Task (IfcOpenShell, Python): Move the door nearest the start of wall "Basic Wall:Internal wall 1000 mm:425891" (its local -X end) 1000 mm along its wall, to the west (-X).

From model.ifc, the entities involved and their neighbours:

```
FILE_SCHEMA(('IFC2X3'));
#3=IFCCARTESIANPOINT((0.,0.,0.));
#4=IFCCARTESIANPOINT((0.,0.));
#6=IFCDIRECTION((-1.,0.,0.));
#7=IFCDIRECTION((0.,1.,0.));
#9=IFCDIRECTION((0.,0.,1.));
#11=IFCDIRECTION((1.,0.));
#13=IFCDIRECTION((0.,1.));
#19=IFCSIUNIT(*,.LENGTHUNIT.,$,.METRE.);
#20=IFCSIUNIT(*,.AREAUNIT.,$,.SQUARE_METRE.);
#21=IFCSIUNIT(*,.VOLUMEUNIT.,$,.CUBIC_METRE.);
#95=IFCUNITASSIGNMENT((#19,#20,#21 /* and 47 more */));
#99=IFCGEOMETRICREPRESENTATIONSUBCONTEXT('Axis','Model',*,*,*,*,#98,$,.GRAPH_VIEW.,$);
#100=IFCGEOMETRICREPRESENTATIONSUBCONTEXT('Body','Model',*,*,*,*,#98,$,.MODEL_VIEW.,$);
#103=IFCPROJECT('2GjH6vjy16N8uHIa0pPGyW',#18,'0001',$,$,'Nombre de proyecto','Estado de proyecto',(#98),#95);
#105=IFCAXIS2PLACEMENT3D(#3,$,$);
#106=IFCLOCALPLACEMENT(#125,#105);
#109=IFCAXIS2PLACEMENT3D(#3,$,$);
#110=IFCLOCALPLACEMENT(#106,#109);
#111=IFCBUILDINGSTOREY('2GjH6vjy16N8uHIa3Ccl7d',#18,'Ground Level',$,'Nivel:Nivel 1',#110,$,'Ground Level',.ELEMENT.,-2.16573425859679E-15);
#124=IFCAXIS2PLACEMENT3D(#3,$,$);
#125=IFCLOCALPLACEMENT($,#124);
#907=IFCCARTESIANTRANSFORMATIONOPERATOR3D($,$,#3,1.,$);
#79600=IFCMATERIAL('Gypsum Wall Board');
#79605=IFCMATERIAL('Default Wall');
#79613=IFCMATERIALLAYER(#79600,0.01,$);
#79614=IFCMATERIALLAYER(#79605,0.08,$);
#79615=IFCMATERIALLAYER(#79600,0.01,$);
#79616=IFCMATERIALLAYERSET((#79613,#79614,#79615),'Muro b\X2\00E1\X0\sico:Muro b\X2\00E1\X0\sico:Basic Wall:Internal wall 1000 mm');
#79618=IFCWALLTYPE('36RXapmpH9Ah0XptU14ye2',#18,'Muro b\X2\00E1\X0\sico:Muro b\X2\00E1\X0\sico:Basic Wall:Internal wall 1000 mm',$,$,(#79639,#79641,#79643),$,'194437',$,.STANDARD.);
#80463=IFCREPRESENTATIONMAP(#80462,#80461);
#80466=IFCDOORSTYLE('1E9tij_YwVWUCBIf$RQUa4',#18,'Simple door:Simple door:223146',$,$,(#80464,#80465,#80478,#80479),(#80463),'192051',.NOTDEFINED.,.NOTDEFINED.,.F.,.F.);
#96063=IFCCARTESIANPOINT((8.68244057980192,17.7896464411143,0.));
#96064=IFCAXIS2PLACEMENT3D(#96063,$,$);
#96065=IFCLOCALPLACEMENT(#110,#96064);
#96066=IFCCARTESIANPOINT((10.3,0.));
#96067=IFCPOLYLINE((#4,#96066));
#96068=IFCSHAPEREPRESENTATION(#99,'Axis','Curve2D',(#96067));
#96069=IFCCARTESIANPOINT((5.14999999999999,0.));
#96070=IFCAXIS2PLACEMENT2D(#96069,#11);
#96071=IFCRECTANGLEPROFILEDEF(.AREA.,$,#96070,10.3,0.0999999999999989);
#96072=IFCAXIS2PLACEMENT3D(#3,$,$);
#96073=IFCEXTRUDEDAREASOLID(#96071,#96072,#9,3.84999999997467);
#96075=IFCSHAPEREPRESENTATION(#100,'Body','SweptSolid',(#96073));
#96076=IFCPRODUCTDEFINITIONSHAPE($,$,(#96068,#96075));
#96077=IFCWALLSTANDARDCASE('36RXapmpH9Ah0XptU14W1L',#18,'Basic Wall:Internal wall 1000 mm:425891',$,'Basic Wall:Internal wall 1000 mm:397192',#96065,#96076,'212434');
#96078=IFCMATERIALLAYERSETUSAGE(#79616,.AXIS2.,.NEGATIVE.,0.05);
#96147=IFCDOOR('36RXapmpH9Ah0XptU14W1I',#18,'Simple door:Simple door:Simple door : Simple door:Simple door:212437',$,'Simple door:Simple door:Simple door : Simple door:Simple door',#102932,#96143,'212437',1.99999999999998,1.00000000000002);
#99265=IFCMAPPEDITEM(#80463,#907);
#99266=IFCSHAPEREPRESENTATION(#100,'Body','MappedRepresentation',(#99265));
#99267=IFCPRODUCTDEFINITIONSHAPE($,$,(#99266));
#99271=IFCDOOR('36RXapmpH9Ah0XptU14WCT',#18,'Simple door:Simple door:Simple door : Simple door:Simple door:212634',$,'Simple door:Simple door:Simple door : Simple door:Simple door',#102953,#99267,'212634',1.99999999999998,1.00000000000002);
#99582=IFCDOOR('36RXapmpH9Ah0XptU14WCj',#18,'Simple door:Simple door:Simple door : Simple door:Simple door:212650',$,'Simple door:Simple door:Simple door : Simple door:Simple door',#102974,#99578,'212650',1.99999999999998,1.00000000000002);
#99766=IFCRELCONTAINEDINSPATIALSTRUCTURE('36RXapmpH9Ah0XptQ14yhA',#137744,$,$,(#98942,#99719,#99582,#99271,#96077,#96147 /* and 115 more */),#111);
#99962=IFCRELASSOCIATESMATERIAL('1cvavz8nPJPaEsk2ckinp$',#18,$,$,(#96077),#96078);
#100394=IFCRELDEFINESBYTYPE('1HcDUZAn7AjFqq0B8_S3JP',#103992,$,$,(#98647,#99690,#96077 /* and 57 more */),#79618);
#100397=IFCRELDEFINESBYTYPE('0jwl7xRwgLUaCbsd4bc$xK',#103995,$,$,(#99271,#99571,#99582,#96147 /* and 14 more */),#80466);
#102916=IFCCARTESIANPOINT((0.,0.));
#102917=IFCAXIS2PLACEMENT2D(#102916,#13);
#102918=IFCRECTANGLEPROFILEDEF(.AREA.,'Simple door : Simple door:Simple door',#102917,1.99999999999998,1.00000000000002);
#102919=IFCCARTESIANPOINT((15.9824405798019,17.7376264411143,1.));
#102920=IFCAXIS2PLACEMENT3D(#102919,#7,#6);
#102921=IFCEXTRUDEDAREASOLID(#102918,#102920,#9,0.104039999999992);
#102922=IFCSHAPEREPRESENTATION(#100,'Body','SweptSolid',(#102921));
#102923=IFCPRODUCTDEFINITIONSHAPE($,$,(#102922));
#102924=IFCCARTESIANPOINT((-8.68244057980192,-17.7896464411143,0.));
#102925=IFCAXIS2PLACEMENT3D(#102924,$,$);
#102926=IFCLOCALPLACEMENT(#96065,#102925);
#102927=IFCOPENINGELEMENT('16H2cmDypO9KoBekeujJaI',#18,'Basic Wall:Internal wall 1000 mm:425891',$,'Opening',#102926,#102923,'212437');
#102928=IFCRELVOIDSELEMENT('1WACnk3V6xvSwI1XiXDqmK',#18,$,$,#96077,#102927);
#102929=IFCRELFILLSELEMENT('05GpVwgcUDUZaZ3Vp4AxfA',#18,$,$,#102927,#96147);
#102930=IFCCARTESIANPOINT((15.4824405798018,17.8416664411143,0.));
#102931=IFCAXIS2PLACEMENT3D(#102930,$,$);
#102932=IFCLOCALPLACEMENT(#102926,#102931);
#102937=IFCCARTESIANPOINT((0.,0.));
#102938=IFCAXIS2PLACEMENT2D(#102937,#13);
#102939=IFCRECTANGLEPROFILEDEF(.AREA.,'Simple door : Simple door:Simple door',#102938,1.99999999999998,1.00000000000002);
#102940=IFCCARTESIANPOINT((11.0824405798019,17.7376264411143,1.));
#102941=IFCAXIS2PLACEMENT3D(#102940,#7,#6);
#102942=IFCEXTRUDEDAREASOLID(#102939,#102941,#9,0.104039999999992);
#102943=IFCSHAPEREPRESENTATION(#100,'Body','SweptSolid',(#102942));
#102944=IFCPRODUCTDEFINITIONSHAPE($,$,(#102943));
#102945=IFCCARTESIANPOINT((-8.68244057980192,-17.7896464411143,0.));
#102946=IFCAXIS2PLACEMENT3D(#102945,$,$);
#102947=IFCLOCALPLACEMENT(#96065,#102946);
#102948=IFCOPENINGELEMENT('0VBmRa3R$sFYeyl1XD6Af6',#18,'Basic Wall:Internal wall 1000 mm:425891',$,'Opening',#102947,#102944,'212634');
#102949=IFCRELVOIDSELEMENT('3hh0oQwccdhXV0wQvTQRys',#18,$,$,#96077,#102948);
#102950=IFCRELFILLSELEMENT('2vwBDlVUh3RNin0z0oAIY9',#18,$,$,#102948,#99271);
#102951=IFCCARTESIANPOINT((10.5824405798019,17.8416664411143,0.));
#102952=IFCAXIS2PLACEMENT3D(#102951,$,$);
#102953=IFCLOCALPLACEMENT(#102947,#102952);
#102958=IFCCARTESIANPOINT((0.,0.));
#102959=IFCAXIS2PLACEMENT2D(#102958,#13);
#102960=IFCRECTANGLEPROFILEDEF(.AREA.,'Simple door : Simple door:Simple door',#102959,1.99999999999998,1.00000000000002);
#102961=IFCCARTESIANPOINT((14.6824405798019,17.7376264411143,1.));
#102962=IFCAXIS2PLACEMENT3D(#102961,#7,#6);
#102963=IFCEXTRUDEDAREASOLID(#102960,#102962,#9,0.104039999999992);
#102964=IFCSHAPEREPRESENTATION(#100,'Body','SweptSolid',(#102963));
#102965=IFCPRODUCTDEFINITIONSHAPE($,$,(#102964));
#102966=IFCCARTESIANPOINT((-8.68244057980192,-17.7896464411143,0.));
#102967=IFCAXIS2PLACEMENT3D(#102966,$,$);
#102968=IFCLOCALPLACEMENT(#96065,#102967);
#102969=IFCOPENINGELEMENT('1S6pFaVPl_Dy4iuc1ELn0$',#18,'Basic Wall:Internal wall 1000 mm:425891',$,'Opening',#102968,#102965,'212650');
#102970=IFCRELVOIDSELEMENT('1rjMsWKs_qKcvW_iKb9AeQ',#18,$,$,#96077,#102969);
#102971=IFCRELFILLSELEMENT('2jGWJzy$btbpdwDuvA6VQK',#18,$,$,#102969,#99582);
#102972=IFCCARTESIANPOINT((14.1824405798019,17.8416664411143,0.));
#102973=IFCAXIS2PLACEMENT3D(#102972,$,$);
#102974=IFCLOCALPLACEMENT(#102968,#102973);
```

```python
import ifcopenshell
import ifcopenshell.api.geometry
import ifcopenshell.util.placement
import ifcopenshell.util.unit

model = ifcopenshell.open("model.ifc")
unit_scale = ifcopenshell.util.unit.calculate_unit_scale(model)

door = model.by_id(99271)
opening = door.FillsVoids[0].RelatingOpeningElement
wall = opening.VoidsElements[0].RelatingBuildingElement

wall_matrix = ifcopenshell.util.placement.get_local_placement(wall.ObjectPlacement)
shift = wall_matrix[:3, 0] * -1 / unit_scale
before = ifcopenshell.util.placement.get_local_placement(door.ObjectPlacement)[:3, 3].copy()

# The door is placed relative to its opening, so it follows when the opening moves.
matrix = ifcopenshell.util.placement.get_local_placement(opening.ObjectPlacement)
matrix[:3, 3] += shift
ifcopenshell.api.geometry.edit_object_placement(
    model, product=opening, matrix=matrix, is_si=False, should_transform_children=True
)

after = ifcopenshell.util.placement.get_local_placement(door.ObjectPlacement)[:3, 3]
print("door moved by", (after - before).round(3) + 0.0)

model.write("model-out.ifc")
```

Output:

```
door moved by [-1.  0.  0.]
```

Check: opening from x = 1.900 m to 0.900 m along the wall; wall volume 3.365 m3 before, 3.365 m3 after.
